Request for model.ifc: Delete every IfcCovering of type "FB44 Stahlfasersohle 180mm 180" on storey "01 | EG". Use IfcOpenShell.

First a look at what the model holds.

```python
import ifcopenshell
import ifcopenshell.util.element

model = ifcopenshell.open("model.ifc")
print(model.schema)
storey = next(s for s in model.by_type("IfcBuildingStorey") if s.Name == "01 | EG")
coverings = [e for e in ifcopenshell.util.element.get_decomposition(storey) if e.is_a("IfcCovering")]
seen = {}
for e in coverings:
    element_type = ifcopenshell.util.element.get_type(e)
    name = element_type.Name if element_type not in (None, e) else None
    seen[name] = seen.get(name, 0) + 1
for name, count in sorted(seen.items(), key=str):
    print(count, "x", name)
```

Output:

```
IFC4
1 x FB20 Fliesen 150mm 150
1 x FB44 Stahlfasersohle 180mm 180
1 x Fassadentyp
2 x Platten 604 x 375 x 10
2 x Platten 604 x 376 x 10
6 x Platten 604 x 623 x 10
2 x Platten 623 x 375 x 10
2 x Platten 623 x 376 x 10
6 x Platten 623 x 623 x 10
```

```python
import ifcopenshell
import ifcopenshell.api.root
import ifcopenshell.util.element

model = ifcopenshell.open("model.ifc")

storey = next(s for s in model.by_type("IfcBuildingStorey") if s.Name == "01 | EG")
coverings = [e for e in ifcopenshell.util.element.get_decomposition(storey) if e.is_a("IfcCovering")]
targets = [e for e in coverings if (t := ifcopenshell.util.element.get_type(e)) not in (None, e) and t.Name == "FB44 Stahlfasersohle 180mm 180"]

for e in targets:
    ifcopenshell.api.root.remove_product(model, product=e)
print(len(targets), "removed")

model.write("model_updated.ifc")
```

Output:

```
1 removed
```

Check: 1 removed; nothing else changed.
